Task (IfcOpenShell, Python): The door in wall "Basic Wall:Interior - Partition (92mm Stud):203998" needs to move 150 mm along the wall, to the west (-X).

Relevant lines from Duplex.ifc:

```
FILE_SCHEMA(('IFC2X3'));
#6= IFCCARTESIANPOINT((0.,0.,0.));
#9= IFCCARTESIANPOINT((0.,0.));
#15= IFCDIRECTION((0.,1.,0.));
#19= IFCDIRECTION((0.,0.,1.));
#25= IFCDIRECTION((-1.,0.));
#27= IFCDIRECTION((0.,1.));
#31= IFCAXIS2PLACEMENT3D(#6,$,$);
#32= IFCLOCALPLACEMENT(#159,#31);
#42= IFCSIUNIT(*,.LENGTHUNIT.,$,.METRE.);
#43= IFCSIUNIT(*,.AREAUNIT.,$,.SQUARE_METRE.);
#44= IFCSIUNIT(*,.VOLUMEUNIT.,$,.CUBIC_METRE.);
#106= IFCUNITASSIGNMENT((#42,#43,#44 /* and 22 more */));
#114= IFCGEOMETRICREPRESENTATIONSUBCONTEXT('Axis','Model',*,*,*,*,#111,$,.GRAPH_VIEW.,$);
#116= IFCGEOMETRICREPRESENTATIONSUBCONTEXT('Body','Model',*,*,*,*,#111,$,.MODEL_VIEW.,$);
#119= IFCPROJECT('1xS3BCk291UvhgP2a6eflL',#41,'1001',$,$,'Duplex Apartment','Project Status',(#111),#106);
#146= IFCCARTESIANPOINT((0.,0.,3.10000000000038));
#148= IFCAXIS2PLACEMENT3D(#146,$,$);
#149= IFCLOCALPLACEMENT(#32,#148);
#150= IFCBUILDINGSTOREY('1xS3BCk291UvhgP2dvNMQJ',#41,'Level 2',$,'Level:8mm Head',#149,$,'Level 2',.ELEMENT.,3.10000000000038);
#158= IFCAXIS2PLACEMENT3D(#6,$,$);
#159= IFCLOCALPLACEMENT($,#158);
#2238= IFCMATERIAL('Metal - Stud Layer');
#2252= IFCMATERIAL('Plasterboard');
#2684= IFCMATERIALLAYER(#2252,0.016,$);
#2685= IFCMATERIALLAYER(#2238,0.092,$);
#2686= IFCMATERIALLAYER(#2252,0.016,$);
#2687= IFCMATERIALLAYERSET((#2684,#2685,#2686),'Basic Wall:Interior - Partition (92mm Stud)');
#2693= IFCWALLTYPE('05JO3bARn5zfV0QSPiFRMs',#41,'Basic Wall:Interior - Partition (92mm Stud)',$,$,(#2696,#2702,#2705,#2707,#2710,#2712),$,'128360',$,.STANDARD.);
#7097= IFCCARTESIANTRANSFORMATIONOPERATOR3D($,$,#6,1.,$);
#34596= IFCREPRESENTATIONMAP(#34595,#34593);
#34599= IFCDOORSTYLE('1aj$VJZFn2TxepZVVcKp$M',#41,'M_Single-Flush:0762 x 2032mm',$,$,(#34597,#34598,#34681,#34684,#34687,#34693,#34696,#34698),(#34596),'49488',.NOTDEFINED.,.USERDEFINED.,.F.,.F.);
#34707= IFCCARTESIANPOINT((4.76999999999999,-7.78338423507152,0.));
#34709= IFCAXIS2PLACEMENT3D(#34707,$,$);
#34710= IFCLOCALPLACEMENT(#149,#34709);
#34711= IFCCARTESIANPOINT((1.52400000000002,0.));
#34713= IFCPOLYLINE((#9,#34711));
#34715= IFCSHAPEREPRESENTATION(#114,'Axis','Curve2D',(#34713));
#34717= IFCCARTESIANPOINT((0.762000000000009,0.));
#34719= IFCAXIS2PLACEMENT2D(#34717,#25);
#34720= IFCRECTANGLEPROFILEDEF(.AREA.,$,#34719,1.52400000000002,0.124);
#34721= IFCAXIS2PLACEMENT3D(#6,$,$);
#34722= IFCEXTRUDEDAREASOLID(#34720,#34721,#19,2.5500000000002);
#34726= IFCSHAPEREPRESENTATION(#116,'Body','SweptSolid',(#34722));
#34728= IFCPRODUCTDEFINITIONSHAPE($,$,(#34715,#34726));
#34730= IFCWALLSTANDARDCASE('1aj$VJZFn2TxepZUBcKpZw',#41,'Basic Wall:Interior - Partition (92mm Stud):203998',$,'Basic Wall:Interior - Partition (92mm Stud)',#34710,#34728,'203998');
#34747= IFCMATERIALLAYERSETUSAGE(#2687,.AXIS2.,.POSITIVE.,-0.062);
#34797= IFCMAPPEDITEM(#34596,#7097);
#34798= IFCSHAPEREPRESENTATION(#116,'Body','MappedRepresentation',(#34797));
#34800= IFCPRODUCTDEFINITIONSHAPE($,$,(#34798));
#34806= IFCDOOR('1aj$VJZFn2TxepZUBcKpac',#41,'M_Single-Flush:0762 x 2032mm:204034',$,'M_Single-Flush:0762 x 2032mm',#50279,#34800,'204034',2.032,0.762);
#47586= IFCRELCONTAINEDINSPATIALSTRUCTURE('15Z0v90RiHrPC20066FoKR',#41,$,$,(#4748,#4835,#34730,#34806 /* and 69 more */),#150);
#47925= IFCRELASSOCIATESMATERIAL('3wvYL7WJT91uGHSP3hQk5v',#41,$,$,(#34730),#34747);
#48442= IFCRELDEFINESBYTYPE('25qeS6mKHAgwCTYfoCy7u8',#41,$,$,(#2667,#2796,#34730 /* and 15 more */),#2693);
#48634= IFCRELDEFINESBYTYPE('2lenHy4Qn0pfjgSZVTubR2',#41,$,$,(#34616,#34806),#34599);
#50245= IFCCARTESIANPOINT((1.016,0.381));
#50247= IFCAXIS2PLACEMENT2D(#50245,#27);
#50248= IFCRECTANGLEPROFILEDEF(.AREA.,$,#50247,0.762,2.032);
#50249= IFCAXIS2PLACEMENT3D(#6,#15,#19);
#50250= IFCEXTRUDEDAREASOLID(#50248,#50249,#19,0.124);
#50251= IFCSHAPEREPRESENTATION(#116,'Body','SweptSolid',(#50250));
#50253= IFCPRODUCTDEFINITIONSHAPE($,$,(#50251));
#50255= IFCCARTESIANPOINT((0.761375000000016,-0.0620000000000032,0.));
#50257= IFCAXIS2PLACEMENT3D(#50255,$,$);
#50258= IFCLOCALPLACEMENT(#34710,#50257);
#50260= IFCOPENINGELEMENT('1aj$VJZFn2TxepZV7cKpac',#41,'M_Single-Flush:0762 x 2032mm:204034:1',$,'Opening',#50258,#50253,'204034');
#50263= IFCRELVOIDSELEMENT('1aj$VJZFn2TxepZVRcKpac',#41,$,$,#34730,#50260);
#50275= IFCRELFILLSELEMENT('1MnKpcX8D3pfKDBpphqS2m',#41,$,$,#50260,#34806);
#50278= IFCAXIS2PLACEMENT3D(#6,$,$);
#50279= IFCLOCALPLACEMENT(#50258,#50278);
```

```python
import ifcopenshell
import ifcopenshell.api.geometry
import ifcopenshell.util.placement

model = ifcopenshell.open("Duplex.ifc")

door = model.by_guid("1aj$VJZFn2TxepZUBcKpac")
opening = door.FillsVoids[0].RelatingOpeningElement
wall = opening.VoidsElements[0].RelatingBuildingElement

wall_matrix = ifcopenshell.util.placement.get_local_placement(wall.ObjectPlacement)
shift = wall_matrix[:3, 0] * -0.15
before = ifcopenshell.util.placement.get_local_placement(door.ObjectPlacement)[:3, 3].copy()

# The door is placed relative to its opening, so it follows when the opening moves.
matrix = ifcopenshell.util.placement.get_local_placement(opening.ObjectPlacement)
matrix[:3, 3] += shift
ifcopenshell.api.geometry.edit_object_placement(
    model, product=opening, matrix=matrix, is_si=False, should_transform_children=True
)

after = ifcopenshell.util.placement.get_local_placement(door.ObjectPlacement)[:3, 3]
print("door moved by", (after - before).round(3) + 0.0)

model.write("Duplex-out.ifc")
```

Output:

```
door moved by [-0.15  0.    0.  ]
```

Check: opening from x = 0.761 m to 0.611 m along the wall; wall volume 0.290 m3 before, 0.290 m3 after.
